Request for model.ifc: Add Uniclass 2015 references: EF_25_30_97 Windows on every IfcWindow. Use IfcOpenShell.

First a look at what the model holds.

```python
import ifcopenshell

model = ifcopenshell.open("model.ifc")
print(model.schema)
print("classifications:", [c.Name for c in model.by_type("IfcClassification")])
for ifc_class in ("IfcDoor", "IfcRoof", "IfcStair", "IfcWall", "IfcWindow"):
    print(ifc_class, len(model.by_type(ifc_class)))
```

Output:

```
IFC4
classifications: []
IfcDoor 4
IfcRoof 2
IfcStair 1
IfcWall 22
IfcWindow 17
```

```python
import ifcopenshell
import ifcopenshell.api.classification

model = ifcopenshell.open("model.ifc")

system = ifcopenshell.api.classification.add_classification(model, classification="Uniclass 2015")

codes = {
    "IfcWindow": ("EF_25_30_97", "Windows"),
}
for ifc_class, (code, name) in codes.items():
    products = model.by_type(ifc_class)
    ifcopenshell.api.classification.add_reference(
        model, products=products, classification=system, identification=code, name=name
    )
    print(code, len(products))

model.write("model_rev.ifc")
```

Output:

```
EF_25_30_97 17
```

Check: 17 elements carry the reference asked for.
